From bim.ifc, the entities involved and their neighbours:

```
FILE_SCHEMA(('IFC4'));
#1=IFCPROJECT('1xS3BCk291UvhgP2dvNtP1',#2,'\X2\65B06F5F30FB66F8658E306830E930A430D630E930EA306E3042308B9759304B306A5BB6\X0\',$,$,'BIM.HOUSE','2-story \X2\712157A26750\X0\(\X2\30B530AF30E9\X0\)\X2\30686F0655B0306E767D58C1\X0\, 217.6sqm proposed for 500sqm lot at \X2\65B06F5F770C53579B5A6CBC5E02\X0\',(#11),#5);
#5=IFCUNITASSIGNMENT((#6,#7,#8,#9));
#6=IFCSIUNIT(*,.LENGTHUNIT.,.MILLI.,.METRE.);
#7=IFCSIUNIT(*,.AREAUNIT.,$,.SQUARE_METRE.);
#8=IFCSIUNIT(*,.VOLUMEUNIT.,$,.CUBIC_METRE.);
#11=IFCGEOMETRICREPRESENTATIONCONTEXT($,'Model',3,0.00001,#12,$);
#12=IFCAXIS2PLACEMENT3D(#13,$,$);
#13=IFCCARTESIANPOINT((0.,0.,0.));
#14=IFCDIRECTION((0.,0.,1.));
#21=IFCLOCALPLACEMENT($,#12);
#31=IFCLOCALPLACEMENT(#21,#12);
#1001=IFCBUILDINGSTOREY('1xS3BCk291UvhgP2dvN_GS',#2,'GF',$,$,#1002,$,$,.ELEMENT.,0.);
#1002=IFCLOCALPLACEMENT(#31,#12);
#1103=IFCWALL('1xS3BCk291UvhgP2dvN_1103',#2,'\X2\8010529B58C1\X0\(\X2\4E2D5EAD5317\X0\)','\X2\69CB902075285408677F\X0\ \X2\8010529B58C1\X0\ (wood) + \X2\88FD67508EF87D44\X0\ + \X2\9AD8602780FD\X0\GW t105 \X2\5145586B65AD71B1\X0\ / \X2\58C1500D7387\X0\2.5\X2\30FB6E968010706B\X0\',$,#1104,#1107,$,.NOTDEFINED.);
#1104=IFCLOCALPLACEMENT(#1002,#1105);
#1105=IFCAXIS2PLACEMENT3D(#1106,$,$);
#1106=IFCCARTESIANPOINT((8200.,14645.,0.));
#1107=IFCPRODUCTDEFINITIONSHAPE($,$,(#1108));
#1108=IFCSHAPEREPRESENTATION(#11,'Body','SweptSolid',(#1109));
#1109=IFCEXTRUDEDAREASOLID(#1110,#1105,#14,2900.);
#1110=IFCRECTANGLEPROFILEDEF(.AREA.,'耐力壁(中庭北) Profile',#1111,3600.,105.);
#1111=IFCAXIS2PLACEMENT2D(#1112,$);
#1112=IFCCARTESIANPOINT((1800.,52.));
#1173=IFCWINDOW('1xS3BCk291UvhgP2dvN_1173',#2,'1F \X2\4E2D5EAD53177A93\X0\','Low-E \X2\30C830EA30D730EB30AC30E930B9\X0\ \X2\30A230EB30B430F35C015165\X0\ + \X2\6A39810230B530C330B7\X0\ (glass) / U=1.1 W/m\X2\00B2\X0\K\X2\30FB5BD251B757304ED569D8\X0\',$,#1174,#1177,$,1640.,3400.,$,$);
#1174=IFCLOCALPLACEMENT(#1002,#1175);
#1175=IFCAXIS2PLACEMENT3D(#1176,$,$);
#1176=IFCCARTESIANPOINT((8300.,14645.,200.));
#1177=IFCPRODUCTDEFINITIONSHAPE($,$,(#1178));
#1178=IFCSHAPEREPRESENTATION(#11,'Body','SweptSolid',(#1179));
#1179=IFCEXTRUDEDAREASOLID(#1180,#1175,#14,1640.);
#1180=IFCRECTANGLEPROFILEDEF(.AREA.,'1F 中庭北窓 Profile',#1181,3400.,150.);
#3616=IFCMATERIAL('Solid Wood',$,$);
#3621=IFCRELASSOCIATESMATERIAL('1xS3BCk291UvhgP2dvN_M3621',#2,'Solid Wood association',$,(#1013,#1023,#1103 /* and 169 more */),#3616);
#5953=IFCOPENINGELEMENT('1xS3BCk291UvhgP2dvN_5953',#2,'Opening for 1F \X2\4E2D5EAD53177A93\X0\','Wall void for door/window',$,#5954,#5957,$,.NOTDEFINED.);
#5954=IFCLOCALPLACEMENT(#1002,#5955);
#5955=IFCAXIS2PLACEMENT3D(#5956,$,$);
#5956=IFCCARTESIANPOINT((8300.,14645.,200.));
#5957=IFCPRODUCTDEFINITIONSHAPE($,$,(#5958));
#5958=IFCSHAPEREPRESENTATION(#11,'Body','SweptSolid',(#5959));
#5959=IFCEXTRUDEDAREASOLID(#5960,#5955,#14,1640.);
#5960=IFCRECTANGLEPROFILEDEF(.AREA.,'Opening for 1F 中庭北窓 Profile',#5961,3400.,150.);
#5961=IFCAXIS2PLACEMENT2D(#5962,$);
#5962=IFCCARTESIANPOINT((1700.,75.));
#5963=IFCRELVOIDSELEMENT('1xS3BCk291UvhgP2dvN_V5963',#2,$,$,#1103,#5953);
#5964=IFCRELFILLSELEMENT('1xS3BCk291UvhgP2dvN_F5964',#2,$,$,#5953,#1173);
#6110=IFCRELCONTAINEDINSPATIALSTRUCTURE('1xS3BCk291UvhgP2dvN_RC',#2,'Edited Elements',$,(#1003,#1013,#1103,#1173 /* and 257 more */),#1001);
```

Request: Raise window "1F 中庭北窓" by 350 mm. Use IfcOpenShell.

```python
import numpy as np
import ifcopenshell
import ifcopenshell.api.geometry
import ifcopenshell.util.placement
import ifcopenshell.util.unit

model = ifcopenshell.open("bim.ifc")
unit_scale = ifcopenshell.util.unit.calculate_unit_scale(model)

window = model.by_id(1173)
opening = window.FillsVoids[0].RelatingOpeningElement
dz = 0.35 / unit_scale

shift = np.array([0.0, 0.0, dz])
# The window is not placed relative to its opening, so move both.
for product in (opening, window):
    matrix = ifcopenshell.util.placement.get_local_placement(product.ObjectPlacement)
    matrix[:3, 3] += shift
    ifcopenshell.api.geometry.edit_object_placement(model, product=product, matrix=matrix, is_si=False)

print(f"moved by {dz * unit_scale:+.3f} m")

model.write("bim_v2.ifc")
```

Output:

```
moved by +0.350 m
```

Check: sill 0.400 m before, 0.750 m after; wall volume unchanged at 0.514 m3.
